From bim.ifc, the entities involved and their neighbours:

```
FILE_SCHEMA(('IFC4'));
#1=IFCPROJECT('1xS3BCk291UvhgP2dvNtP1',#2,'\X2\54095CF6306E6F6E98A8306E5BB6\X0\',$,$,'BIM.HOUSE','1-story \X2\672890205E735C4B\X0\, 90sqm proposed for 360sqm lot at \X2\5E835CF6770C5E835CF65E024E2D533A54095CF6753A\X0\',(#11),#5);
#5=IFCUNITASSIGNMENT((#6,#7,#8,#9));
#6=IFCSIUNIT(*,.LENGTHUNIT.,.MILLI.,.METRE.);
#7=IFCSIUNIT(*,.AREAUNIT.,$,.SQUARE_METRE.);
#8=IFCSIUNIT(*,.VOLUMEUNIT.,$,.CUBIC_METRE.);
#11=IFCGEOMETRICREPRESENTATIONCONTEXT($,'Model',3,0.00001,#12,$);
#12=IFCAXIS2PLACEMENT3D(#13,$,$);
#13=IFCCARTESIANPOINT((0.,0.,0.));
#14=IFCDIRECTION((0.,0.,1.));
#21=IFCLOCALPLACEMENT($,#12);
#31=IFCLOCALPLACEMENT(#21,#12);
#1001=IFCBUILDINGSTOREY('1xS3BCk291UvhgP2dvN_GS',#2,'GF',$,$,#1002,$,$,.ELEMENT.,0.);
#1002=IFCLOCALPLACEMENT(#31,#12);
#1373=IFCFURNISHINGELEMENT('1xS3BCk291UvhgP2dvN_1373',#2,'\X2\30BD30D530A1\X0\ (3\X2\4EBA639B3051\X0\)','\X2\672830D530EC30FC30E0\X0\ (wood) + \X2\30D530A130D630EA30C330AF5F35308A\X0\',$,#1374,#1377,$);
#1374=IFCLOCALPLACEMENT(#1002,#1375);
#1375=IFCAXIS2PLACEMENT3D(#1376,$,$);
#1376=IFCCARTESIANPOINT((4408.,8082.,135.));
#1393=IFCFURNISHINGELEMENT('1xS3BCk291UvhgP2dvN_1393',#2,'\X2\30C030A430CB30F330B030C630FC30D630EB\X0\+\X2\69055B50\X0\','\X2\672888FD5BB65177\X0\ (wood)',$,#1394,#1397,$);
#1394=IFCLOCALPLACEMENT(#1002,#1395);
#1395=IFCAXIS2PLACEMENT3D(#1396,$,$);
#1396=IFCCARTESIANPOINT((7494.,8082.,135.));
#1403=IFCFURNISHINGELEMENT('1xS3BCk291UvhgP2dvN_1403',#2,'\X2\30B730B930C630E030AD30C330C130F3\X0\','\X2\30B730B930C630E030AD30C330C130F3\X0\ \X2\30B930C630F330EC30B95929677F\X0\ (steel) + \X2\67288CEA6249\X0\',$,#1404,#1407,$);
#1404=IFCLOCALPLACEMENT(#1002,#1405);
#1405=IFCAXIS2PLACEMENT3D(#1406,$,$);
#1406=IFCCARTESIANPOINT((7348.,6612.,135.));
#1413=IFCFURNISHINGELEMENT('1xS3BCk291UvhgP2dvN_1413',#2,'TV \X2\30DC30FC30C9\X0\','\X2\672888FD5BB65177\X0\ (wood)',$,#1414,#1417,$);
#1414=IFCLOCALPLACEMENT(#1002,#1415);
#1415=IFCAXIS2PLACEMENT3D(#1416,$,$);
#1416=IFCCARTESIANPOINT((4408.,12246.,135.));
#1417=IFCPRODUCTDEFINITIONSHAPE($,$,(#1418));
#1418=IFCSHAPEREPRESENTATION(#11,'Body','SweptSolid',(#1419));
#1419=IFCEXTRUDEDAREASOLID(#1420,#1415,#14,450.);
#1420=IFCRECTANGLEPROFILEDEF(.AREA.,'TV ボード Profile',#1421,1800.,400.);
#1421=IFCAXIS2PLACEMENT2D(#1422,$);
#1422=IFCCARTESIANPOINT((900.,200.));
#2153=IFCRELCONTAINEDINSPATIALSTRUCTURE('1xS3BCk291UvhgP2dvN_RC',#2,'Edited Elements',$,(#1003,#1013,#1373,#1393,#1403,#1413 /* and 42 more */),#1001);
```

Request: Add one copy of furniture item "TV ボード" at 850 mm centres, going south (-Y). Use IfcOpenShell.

```python
import numpy as np
import ifcopenshell
import ifcopenshell.api.geometry
import ifcopenshell.api.root
import ifcopenshell.util.element
import ifcopenshell.util.placement
import ifcopenshell.util.unit

model = ifcopenshell.open("bim.ifc")
unit_scale = ifcopenshell.util.unit.calculate_unit_scale(model)


def reuse_history(source, copy):
    """copy_class also copies each property set's owner history, people and application; keep the originals."""
    for rel in copy.IsDefinedBy:
        if rel.is_a("IfcRelDefinesByProperties") and (history := rel.RelatingPropertyDefinition.OwnerHistory):
            rel.RelatingPropertyDefinition.OwnerHistory = source.OwnerHistory
            ifcopenshell.util.element.remove_deep2(model, history)


source = model.by_guid("1xS3BCk291UvhgP2dvN_1413")
base = ifcopenshell.util.placement.get_local_placement(source.ObjectPlacement)
step = np.array([0.0, -1.0, 0.0]) * 0.85 / unit_scale

for i in range(1, 2):
    copy = ifcopenshell.api.root.copy_class(model, product=source)
    copy.Representation = ifcopenshell.util.element.copy_deep(
        model, source.Representation, exclude=["IfcGeometricRepresentationContext", "IfcRepresentationMap"]
    )
    reuse_history(source, copy)
    matrix = base.copy()
    matrix[:3, 3] += i * step
    print("added at", matrix[:3, 3].round(3) + 0.0)
    ifcopenshell.api.geometry.edit_object_placement(model, product=copy, matrix=matrix, is_si=False)

model.write("bim-out.ifc")
```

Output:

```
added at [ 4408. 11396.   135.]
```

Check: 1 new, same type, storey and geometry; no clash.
